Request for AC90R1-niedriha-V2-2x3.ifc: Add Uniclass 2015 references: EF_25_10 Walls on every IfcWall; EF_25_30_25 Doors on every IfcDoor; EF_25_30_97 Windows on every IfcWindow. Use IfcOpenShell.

First a look at what the model holds.

```python
import ifcopenshell

model = ifcopenshell.open("AC90R1-niedriha-V2-2x3.ifc")
print(model.schema)
print("classifications:", [c.Name for c in model.by_type("IfcClassification")])
for ifc_class in ("IfcDoor", "IfcRoof", "IfcStair", "IfcWall", "IfcWindow"):
    print(ifc_class, len(model.by_type(ifc_class)))
```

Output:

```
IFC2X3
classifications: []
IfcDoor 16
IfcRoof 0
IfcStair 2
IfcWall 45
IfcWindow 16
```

```python
import ifcopenshell
import ifcopenshell.api.classification

model = ifcopenshell.open("AC90R1-niedriha-V2-2x3.ifc")

# IFC2X3 requires Source and Edition and has no link from the project to the system.
system = model.create_entity("IfcClassification", Source="NBS", Edition="2015", Name="Uniclass 2015")

codes = {
    "IfcWall": ("EF_25_10", "Walls"),
    "IfcDoor": ("EF_25_30_25", "Doors"),
    "IfcWindow": ("EF_25_30_97", "Windows"),
}
for ifc_class, (code, name) in codes.items():
    products = model.by_type(ifc_class)
    ifcopenshell.api.classification.add_reference(
        model, products=products, classification=system, identification=code, name=name
    )
    print(code, len(products))

model.write("AC90R1-niedriha-V2-2x3-out.ifc")
```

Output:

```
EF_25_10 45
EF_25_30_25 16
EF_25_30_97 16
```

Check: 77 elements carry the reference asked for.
